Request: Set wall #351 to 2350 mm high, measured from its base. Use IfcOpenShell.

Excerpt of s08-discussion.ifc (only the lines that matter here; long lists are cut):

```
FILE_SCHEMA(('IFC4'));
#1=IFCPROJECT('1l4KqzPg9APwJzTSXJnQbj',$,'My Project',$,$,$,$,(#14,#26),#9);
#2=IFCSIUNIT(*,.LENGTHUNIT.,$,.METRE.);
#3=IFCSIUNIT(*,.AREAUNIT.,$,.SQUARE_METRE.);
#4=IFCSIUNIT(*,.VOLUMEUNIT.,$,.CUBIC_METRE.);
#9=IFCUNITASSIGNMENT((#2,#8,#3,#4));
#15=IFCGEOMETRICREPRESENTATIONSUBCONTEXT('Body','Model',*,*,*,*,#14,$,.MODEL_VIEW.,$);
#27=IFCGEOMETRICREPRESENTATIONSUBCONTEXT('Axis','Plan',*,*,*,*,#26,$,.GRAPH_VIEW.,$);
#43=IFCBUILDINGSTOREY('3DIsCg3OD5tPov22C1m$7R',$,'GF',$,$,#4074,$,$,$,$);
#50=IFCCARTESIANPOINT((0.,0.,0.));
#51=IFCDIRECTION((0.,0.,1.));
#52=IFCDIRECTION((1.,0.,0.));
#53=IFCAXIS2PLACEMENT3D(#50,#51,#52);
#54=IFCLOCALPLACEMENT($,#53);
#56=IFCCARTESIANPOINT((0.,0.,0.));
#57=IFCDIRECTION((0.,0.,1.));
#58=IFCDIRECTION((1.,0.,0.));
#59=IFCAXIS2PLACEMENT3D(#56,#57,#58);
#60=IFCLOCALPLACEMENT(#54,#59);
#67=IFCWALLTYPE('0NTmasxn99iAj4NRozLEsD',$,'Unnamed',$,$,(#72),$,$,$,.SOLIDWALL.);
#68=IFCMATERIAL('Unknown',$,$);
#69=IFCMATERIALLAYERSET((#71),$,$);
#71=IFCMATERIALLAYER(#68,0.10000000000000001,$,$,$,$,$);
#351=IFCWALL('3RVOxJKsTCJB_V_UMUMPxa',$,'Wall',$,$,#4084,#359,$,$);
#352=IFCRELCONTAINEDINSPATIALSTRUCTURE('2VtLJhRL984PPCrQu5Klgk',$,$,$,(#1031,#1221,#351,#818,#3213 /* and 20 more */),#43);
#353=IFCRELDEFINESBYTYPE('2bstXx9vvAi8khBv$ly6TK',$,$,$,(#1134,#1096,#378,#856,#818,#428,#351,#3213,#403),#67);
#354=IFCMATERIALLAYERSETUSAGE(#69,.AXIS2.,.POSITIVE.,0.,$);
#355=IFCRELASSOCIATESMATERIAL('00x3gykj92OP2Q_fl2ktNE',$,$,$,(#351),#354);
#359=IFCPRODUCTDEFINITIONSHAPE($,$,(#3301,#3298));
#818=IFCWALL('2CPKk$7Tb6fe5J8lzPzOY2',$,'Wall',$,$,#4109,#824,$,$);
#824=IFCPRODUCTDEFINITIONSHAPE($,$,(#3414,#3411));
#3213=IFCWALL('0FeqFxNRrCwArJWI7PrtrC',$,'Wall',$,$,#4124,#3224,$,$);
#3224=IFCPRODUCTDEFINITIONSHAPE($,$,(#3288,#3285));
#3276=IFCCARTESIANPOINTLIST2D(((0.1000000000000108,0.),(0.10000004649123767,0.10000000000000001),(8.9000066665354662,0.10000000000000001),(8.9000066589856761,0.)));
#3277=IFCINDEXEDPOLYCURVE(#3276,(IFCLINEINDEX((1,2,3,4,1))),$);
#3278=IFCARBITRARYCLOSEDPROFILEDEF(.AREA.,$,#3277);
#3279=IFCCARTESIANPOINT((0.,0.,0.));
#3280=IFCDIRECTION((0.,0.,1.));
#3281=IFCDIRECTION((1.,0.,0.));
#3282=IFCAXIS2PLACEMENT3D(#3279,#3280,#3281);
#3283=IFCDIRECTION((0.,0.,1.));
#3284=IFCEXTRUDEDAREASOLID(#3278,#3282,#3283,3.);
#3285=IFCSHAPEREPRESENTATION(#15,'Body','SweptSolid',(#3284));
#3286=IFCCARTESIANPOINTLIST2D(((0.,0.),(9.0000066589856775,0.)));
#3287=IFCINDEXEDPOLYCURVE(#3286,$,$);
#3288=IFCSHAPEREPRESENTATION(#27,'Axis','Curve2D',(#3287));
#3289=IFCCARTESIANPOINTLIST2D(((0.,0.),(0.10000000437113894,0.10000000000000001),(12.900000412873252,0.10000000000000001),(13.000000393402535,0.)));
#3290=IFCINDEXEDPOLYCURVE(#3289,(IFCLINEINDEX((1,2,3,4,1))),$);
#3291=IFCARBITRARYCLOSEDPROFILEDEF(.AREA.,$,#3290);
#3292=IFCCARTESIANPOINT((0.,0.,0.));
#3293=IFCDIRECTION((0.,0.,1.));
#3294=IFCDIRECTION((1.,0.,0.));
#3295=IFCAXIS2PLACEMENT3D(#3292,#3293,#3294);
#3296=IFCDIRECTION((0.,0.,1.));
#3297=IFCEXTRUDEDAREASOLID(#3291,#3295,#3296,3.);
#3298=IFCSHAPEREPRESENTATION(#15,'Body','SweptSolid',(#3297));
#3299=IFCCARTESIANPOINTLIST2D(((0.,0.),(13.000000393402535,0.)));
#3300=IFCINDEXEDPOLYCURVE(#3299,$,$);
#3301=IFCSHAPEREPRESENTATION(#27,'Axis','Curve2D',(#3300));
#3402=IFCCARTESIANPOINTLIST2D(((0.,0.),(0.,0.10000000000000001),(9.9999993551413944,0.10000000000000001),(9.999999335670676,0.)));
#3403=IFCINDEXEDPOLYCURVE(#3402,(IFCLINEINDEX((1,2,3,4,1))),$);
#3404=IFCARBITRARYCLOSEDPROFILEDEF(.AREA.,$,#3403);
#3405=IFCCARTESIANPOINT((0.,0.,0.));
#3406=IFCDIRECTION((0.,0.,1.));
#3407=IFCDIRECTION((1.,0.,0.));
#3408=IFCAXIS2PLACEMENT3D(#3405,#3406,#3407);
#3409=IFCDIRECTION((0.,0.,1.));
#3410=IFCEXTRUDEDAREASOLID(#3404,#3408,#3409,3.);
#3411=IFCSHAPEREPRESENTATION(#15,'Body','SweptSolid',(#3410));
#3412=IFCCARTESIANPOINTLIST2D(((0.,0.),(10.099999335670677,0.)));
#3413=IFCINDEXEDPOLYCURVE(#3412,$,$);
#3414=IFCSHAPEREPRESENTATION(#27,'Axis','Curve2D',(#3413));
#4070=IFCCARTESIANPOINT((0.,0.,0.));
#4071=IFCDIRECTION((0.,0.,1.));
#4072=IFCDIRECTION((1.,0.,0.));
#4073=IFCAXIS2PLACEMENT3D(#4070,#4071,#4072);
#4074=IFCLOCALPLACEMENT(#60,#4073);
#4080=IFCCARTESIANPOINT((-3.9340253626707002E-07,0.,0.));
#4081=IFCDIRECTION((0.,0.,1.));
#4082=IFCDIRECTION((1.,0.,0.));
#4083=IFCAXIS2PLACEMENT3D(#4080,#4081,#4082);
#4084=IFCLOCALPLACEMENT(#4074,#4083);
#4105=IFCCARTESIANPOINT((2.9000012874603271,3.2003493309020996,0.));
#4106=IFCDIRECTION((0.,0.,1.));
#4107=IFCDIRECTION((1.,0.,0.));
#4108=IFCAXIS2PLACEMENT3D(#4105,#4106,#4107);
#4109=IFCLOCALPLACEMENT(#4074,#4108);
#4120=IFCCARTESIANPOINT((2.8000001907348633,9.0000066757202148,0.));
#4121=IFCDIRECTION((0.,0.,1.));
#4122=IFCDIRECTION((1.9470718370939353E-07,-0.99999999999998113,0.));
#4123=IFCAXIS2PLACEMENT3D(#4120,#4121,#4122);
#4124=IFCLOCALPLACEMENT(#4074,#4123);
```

```python
import ifcopenshell
import ifcopenshell.geom
import ifcopenshell.util.representation
import ifcopenshell.util.shape

model = ifcopenshell.open("s08-discussion.ifc")
settings = ifcopenshell.geom.settings()


def volume(element):
    """Net volume in cubic metres, openings subtracted."""
    shape = ifcopenshell.geom.create_shape(settings, element)
    return ifcopenshell.util.shape.get_volume(shape.geometry)


wall = model.by_guid("3RVOxJKsTCJB_V_UMUMPxa")
before = volume(wall)

body = ifcopenshell.util.representation.get_representation(wall, "Model", "Body")
solid = body.Items[0]
old_height = solid.Depth
solid.Depth = 2.35
after = volume(wall)

print(f"height {old_height:g} -> {solid.Depth:g}, volume {before:.3f} -> {after:.3f} m3")

model.write("s08-discussion-out.ifc")
```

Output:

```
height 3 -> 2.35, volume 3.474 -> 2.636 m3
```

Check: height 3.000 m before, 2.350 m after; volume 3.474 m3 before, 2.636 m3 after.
